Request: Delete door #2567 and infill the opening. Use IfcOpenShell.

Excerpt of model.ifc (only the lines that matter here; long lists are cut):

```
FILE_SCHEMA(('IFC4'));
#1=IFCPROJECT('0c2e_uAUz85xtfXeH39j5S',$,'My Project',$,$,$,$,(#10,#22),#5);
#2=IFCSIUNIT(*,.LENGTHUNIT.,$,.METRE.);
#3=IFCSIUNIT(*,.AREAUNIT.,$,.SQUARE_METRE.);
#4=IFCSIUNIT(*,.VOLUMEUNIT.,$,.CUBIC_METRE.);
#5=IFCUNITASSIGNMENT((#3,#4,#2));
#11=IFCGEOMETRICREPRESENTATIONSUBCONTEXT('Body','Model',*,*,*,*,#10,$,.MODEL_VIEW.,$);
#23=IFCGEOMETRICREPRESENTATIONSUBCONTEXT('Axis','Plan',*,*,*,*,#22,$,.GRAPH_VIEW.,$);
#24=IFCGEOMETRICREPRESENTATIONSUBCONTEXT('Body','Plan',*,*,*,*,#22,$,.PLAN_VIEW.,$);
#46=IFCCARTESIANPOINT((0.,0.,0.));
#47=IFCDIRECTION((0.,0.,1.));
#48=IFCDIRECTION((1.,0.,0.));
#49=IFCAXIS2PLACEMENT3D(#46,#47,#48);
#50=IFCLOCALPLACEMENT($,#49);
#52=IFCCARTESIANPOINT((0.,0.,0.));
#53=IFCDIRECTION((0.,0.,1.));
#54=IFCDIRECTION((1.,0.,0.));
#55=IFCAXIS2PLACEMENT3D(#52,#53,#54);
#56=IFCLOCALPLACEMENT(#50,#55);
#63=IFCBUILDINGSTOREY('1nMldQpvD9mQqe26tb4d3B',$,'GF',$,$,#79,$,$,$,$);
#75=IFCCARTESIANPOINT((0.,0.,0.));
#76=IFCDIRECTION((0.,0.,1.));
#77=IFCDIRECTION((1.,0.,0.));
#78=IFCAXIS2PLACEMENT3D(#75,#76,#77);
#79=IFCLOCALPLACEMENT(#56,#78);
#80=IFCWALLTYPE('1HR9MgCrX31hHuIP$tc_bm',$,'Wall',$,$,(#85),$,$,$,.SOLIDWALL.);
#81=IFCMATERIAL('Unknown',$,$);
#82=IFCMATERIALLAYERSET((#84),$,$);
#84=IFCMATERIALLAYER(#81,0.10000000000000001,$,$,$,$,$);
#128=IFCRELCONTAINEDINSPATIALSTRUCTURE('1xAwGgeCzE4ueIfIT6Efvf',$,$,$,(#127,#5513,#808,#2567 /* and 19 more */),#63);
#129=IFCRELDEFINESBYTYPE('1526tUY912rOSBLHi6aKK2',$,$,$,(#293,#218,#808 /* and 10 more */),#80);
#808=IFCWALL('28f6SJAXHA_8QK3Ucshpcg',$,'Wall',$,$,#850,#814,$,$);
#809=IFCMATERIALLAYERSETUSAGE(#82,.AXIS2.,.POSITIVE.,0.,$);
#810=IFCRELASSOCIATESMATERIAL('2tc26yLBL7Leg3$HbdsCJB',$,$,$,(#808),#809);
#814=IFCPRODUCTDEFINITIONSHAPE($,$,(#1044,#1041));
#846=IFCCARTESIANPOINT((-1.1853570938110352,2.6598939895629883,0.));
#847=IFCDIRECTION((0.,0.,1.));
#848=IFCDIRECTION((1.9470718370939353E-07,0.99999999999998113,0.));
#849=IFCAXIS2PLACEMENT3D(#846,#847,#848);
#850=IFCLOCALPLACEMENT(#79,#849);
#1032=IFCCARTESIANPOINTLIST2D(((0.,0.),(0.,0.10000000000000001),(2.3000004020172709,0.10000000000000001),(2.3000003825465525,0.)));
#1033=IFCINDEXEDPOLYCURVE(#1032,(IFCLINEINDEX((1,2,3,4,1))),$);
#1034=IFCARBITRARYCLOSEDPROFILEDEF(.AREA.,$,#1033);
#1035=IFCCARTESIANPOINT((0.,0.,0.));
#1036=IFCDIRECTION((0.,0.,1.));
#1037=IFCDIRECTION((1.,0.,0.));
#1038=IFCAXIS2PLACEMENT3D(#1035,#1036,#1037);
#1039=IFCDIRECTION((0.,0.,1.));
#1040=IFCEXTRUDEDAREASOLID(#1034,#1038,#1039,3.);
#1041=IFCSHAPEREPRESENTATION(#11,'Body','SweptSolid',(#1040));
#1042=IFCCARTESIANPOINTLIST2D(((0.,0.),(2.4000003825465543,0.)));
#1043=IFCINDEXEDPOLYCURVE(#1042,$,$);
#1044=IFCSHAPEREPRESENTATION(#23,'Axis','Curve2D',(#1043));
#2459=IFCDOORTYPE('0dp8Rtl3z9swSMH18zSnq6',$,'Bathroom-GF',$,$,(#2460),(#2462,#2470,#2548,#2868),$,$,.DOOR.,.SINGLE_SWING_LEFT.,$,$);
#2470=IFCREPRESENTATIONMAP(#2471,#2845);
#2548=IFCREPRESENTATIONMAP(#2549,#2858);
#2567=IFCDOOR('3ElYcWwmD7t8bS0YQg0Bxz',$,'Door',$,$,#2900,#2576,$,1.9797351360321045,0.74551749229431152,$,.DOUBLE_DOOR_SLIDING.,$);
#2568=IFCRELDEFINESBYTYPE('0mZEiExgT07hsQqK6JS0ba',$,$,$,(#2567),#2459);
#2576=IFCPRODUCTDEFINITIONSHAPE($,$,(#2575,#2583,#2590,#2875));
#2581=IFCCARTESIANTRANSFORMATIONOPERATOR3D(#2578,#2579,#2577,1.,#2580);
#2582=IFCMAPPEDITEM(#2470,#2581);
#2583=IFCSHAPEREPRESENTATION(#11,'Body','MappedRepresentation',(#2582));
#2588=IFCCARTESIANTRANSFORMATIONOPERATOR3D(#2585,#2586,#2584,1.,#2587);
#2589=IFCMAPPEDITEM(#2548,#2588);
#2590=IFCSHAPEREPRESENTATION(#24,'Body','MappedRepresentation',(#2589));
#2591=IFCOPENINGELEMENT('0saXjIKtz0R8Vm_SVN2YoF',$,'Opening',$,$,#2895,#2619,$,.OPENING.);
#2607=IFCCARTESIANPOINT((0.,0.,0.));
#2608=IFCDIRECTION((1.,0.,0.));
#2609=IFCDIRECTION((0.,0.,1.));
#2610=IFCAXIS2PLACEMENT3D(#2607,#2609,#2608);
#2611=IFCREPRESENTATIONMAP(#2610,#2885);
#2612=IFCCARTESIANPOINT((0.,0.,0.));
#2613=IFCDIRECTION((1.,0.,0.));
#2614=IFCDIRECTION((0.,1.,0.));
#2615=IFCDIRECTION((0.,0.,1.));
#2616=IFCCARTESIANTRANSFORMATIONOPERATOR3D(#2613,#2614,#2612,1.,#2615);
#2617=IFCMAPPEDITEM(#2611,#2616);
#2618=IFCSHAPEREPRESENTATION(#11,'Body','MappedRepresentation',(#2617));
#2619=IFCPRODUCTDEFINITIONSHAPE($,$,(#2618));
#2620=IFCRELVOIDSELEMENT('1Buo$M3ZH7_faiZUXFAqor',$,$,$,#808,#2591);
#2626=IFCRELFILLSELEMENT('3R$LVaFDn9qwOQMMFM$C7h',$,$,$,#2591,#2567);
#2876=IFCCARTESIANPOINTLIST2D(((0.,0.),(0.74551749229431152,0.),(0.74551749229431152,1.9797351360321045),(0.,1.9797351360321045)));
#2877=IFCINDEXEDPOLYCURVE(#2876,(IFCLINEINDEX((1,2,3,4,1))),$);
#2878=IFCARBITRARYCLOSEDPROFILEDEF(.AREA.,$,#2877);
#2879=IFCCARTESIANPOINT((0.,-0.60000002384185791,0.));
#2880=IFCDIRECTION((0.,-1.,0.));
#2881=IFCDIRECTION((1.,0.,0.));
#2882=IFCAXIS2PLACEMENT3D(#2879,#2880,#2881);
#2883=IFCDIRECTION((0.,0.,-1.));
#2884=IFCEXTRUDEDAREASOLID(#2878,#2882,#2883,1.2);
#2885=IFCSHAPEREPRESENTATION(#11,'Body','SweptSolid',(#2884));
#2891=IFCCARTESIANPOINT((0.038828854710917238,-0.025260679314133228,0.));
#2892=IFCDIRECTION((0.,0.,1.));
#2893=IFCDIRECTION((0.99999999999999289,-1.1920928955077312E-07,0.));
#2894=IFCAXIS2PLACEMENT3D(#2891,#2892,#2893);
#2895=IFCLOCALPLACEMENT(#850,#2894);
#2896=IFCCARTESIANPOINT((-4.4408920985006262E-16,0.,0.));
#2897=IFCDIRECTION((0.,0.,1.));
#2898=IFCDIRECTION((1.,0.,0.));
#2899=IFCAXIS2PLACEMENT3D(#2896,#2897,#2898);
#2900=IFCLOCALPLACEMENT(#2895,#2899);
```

```python
import ifcopenshell
import ifcopenshell.api.feature
import ifcopenshell.api.root
import ifcopenshell.geom
import ifcopenshell.util.shape

model = ifcopenshell.open("model.ifc")
settings = ifcopenshell.geom.settings()


def volume(element):
    """Net volume in cubic metres, openings subtracted."""
    shape = ifcopenshell.geom.create_shape(settings, element)
    return ifcopenshell.util.shape.get_volume(shape.geometry)


door = model.by_guid("3ElYcWwmD7t8bS0YQg0Bxz")
opening = door.FillsVoids[0].RelatingOpeningElement
wall = opening.VoidsElements[0].RelatingBuildingElement
before = volume(wall)

ifcopenshell.api.root.remove_product(model, product=door)
ifcopenshell.api.feature.remove_feature(model, feature=opening)

after = volume(wall)

print(f"wall volume {before:.3f} -> {after:.3f} m3")

model.write("model_edited.ifc")
```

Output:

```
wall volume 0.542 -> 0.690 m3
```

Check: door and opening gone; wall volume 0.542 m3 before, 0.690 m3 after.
